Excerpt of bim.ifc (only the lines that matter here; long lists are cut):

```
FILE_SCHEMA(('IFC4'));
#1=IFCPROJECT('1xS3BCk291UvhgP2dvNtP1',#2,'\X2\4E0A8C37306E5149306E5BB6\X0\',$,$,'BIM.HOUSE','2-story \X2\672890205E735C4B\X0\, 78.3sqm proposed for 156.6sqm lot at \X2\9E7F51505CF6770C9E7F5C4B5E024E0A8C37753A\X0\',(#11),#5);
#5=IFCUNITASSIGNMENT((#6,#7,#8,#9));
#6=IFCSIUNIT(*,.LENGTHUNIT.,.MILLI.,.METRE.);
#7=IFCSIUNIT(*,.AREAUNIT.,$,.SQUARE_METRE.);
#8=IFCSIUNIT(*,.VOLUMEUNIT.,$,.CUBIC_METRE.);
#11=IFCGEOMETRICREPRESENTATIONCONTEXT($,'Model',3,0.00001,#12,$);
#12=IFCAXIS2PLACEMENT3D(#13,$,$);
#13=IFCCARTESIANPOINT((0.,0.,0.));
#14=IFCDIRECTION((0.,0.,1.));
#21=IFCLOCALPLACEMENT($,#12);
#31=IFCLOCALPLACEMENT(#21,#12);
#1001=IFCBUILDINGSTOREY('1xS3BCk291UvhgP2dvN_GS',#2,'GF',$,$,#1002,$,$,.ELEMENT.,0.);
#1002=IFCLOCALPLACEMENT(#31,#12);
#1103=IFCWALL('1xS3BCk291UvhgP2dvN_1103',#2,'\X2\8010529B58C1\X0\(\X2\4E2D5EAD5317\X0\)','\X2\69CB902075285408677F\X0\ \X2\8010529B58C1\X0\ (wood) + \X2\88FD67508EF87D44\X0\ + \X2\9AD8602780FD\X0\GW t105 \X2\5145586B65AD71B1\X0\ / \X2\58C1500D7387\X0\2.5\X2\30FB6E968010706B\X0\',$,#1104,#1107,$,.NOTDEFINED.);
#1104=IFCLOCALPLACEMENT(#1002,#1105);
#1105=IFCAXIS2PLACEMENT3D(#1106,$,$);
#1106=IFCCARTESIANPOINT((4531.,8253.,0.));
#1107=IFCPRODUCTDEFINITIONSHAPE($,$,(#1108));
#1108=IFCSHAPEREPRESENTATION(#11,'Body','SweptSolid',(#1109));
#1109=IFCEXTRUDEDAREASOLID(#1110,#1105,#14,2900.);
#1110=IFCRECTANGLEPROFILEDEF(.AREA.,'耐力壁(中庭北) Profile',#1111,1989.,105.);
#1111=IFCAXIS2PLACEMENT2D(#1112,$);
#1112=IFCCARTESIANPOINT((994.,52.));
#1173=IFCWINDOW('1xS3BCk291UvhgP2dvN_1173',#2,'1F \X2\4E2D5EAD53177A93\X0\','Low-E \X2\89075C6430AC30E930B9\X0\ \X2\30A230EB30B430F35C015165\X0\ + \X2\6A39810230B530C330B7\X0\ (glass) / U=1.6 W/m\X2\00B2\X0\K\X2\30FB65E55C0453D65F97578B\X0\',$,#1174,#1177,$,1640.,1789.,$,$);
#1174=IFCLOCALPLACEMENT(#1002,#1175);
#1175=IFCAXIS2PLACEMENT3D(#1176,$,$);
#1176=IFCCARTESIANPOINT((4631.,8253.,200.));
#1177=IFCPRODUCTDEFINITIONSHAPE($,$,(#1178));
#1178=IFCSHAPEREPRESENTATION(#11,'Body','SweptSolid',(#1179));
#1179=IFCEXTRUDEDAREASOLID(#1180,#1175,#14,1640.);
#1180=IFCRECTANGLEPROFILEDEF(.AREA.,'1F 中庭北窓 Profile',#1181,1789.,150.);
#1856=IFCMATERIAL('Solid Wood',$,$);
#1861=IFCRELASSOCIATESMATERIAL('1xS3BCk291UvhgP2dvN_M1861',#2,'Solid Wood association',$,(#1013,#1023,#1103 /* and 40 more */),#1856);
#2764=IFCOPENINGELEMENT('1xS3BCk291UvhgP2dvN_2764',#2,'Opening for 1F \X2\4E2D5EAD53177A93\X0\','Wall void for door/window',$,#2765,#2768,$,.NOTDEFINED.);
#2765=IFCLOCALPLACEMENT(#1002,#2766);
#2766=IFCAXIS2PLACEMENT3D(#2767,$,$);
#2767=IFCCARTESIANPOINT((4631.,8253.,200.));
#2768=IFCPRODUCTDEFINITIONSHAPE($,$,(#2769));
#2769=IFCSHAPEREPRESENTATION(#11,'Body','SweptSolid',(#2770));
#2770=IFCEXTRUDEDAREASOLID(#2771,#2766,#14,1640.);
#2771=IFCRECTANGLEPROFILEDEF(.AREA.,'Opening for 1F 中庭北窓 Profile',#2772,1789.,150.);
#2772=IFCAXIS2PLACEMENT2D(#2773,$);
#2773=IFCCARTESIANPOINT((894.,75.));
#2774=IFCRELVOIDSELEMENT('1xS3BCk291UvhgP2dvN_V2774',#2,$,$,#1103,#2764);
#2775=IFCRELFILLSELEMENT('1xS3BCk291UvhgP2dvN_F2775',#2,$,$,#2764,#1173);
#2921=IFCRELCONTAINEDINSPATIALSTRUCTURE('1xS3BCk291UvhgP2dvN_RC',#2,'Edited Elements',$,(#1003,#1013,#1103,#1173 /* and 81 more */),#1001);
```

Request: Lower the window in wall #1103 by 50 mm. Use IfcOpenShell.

```python
import numpy as np
import ifcopenshell
import ifcopenshell.api.geometry
import ifcopenshell.util.placement
import ifcopenshell.util.unit

model = ifcopenshell.open("bim.ifc")
unit_scale = ifcopenshell.util.unit.calculate_unit_scale(model)

window = model.by_guid("1xS3BCk291UvhgP2dvN_1173")
opening = window.FillsVoids[0].RelatingOpeningElement
dz = -50.0

shift = np.array([0.0, 0.0, dz])
# The window is not placed relative to its opening, so move both.
for product in (opening, window):
    matrix = ifcopenshell.util.placement.get_local_placement(product.ObjectPlacement)
    matrix[:3, 3] += shift
    ifcopenshell.api.geometry.edit_object_placement(model, product=product, matrix=matrix, is_si=False)

print(f"moved by {dz * unit_scale:+.3f} m")

model.write("bim_v2.ifc")
```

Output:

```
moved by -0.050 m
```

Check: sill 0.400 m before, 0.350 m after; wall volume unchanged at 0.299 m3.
